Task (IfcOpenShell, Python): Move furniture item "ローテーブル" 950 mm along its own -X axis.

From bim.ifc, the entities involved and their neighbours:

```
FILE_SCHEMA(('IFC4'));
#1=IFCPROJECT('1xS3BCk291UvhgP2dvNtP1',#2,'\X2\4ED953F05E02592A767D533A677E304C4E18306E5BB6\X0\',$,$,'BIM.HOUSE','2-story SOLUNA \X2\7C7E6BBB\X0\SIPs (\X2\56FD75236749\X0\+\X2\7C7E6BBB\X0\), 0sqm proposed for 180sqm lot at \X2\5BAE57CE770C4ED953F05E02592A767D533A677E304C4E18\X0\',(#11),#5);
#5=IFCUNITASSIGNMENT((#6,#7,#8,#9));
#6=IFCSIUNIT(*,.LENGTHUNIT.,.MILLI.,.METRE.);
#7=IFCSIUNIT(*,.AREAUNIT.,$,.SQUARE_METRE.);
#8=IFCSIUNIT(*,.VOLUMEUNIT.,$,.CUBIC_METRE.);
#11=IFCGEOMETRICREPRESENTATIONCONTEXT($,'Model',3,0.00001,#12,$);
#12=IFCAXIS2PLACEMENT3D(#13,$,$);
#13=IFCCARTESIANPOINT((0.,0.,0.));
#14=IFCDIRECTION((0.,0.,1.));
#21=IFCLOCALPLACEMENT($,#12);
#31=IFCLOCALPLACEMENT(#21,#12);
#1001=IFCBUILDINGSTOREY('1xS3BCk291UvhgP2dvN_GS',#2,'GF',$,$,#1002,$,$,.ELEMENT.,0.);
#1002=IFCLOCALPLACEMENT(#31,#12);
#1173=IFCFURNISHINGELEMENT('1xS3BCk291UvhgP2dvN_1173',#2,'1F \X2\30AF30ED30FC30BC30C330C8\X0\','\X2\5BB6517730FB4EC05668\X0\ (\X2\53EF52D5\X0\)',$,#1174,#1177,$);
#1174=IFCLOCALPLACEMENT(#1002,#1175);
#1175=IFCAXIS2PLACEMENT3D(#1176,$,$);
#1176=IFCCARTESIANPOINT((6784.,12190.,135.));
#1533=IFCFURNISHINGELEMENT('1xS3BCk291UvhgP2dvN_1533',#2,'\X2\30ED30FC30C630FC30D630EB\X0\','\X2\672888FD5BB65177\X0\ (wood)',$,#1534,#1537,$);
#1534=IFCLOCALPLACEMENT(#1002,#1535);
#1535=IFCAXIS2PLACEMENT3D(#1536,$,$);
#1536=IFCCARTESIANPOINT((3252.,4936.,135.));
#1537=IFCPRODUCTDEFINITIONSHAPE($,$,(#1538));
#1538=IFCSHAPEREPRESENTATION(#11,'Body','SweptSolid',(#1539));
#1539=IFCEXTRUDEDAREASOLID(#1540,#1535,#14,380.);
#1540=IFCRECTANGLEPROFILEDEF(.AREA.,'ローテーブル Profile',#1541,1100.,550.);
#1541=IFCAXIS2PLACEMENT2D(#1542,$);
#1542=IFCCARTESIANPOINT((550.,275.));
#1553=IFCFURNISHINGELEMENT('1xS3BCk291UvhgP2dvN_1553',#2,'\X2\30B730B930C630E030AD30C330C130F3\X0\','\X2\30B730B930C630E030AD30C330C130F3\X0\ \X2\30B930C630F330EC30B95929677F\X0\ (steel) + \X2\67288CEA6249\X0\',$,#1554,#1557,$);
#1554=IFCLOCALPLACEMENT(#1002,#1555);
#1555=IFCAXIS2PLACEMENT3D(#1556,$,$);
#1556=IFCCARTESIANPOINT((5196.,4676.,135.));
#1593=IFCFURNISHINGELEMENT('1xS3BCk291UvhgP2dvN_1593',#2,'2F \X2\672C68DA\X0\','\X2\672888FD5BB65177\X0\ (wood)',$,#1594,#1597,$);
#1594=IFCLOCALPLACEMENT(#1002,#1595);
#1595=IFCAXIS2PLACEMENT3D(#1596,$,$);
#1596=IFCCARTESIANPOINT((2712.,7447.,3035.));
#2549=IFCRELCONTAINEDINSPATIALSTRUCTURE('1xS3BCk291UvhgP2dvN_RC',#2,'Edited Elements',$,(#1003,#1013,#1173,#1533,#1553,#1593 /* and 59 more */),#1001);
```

```python
import ifcopenshell
import ifcopenshell.api.geometry
import ifcopenshell.util.placement
import ifcopenshell.util.unit

model = ifcopenshell.open("bim.ifc")
unit_scale = ifcopenshell.util.unit.calculate_unit_scale(model)

item = model.by_guid("1xS3BCk291UvhgP2dvN_1533")
matrix = ifcopenshell.util.placement.get_local_placement(item.ObjectPlacement)
matrix[:3, 3] -= matrix[:3, 0] * 0.95 / unit_scale
ifcopenshell.api.geometry.edit_object_placement(model, product=item, matrix=matrix, is_si=False)

print(ifcopenshell.util.placement.get_local_placement(item.ObjectPlacement).round(3) + 0.0)

model.write("bim_rev.ifc")
```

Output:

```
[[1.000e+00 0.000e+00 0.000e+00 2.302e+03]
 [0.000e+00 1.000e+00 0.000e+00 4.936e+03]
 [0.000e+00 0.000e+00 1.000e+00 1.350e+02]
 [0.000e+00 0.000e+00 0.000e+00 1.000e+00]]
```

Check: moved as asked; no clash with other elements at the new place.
